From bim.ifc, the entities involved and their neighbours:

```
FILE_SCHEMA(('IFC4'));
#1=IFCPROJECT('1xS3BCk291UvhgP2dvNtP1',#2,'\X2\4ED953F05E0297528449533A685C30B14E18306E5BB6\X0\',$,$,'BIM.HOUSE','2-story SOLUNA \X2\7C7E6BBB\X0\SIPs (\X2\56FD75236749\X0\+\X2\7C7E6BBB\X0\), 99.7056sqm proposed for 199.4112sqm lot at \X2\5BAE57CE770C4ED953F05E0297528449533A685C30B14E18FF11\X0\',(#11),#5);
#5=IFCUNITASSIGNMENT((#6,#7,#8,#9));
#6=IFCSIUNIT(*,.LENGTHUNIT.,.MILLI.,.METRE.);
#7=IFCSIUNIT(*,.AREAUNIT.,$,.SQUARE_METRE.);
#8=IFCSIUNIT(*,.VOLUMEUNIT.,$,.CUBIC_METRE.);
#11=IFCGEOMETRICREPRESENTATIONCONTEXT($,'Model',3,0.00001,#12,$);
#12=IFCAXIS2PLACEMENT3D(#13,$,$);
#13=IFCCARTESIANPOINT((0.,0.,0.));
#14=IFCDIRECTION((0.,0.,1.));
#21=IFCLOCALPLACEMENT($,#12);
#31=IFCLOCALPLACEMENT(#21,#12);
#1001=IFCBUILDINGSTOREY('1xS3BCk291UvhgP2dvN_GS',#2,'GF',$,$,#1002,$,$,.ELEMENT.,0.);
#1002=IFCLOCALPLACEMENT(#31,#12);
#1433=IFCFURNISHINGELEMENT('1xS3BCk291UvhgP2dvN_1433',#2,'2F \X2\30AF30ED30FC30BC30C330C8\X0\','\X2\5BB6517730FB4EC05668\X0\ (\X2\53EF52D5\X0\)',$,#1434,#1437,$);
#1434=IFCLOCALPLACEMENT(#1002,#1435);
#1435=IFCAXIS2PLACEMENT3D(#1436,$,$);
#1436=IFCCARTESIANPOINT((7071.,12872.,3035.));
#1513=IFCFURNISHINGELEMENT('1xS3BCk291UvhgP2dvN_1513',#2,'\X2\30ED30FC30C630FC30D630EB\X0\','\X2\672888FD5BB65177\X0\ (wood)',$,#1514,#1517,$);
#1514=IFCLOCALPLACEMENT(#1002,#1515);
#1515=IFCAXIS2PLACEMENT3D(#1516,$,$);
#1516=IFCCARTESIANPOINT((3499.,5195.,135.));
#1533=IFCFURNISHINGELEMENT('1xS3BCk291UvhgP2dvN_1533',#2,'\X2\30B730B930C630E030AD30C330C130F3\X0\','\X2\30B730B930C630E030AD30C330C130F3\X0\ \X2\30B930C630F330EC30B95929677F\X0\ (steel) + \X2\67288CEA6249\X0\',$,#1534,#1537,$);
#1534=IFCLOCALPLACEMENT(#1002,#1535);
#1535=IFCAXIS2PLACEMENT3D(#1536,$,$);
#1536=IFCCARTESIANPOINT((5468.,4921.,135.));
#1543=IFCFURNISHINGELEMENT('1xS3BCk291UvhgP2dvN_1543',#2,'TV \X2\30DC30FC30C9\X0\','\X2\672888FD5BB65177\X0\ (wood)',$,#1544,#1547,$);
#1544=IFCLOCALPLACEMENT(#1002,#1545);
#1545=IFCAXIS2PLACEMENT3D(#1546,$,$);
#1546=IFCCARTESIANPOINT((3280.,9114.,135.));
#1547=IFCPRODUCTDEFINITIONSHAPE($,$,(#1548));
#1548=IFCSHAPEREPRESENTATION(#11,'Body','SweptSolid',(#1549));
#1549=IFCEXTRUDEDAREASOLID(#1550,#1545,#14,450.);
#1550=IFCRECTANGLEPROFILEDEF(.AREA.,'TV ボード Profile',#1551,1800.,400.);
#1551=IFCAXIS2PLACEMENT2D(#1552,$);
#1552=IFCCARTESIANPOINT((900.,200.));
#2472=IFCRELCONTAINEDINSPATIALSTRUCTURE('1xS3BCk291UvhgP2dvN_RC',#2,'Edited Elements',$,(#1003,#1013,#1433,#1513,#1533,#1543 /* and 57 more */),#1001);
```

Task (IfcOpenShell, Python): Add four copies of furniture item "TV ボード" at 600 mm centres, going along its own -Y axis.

```python
import ifcopenshell
import ifcopenshell.api.geometry
import ifcopenshell.api.root
import ifcopenshell.util.element
import ifcopenshell.util.placement
import ifcopenshell.util.unit

model = ifcopenshell.open("bim.ifc")
unit_scale = ifcopenshell.util.unit.calculate_unit_scale(model)


def reuse_history(source, copy):
    """copy_class also copies each property set's owner history, people and application; keep the originals."""
    for rel in copy.IsDefinedBy:
        if rel.is_a("IfcRelDefinesByProperties") and (history := rel.RelatingPropertyDefinition.OwnerHistory):
            rel.RelatingPropertyDefinition.OwnerHistory = source.OwnerHistory
            ifcopenshell.util.element.remove_deep2(model, history)


source = model.by_guid("1xS3BCk291UvhgP2dvN_1543")
base = ifcopenshell.util.placement.get_local_placement(source.ObjectPlacement)
step = -base[:3, 1] * 0.6 / unit_scale

for i in range(1, 5):
    copy = ifcopenshell.api.root.copy_class(model, product=source)
    copy.Representation = ifcopenshell.util.element.copy_deep(
        model, source.Representation, exclude=["IfcGeometricRepresentationContext", "IfcRepresentationMap"]
    )
    reuse_history(source, copy)
    matrix = base.copy()
    matrix[:3, 3] += i * step
    print("added at", matrix[:3, 3].round(3) + 0.0)
    ifcopenshell.api.geometry.edit_object_placement(model, product=copy, matrix=matrix, is_si=False)

model.write("bim-out.ifc")
```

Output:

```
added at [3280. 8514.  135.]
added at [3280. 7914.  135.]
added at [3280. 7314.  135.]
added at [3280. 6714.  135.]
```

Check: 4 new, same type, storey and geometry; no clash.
